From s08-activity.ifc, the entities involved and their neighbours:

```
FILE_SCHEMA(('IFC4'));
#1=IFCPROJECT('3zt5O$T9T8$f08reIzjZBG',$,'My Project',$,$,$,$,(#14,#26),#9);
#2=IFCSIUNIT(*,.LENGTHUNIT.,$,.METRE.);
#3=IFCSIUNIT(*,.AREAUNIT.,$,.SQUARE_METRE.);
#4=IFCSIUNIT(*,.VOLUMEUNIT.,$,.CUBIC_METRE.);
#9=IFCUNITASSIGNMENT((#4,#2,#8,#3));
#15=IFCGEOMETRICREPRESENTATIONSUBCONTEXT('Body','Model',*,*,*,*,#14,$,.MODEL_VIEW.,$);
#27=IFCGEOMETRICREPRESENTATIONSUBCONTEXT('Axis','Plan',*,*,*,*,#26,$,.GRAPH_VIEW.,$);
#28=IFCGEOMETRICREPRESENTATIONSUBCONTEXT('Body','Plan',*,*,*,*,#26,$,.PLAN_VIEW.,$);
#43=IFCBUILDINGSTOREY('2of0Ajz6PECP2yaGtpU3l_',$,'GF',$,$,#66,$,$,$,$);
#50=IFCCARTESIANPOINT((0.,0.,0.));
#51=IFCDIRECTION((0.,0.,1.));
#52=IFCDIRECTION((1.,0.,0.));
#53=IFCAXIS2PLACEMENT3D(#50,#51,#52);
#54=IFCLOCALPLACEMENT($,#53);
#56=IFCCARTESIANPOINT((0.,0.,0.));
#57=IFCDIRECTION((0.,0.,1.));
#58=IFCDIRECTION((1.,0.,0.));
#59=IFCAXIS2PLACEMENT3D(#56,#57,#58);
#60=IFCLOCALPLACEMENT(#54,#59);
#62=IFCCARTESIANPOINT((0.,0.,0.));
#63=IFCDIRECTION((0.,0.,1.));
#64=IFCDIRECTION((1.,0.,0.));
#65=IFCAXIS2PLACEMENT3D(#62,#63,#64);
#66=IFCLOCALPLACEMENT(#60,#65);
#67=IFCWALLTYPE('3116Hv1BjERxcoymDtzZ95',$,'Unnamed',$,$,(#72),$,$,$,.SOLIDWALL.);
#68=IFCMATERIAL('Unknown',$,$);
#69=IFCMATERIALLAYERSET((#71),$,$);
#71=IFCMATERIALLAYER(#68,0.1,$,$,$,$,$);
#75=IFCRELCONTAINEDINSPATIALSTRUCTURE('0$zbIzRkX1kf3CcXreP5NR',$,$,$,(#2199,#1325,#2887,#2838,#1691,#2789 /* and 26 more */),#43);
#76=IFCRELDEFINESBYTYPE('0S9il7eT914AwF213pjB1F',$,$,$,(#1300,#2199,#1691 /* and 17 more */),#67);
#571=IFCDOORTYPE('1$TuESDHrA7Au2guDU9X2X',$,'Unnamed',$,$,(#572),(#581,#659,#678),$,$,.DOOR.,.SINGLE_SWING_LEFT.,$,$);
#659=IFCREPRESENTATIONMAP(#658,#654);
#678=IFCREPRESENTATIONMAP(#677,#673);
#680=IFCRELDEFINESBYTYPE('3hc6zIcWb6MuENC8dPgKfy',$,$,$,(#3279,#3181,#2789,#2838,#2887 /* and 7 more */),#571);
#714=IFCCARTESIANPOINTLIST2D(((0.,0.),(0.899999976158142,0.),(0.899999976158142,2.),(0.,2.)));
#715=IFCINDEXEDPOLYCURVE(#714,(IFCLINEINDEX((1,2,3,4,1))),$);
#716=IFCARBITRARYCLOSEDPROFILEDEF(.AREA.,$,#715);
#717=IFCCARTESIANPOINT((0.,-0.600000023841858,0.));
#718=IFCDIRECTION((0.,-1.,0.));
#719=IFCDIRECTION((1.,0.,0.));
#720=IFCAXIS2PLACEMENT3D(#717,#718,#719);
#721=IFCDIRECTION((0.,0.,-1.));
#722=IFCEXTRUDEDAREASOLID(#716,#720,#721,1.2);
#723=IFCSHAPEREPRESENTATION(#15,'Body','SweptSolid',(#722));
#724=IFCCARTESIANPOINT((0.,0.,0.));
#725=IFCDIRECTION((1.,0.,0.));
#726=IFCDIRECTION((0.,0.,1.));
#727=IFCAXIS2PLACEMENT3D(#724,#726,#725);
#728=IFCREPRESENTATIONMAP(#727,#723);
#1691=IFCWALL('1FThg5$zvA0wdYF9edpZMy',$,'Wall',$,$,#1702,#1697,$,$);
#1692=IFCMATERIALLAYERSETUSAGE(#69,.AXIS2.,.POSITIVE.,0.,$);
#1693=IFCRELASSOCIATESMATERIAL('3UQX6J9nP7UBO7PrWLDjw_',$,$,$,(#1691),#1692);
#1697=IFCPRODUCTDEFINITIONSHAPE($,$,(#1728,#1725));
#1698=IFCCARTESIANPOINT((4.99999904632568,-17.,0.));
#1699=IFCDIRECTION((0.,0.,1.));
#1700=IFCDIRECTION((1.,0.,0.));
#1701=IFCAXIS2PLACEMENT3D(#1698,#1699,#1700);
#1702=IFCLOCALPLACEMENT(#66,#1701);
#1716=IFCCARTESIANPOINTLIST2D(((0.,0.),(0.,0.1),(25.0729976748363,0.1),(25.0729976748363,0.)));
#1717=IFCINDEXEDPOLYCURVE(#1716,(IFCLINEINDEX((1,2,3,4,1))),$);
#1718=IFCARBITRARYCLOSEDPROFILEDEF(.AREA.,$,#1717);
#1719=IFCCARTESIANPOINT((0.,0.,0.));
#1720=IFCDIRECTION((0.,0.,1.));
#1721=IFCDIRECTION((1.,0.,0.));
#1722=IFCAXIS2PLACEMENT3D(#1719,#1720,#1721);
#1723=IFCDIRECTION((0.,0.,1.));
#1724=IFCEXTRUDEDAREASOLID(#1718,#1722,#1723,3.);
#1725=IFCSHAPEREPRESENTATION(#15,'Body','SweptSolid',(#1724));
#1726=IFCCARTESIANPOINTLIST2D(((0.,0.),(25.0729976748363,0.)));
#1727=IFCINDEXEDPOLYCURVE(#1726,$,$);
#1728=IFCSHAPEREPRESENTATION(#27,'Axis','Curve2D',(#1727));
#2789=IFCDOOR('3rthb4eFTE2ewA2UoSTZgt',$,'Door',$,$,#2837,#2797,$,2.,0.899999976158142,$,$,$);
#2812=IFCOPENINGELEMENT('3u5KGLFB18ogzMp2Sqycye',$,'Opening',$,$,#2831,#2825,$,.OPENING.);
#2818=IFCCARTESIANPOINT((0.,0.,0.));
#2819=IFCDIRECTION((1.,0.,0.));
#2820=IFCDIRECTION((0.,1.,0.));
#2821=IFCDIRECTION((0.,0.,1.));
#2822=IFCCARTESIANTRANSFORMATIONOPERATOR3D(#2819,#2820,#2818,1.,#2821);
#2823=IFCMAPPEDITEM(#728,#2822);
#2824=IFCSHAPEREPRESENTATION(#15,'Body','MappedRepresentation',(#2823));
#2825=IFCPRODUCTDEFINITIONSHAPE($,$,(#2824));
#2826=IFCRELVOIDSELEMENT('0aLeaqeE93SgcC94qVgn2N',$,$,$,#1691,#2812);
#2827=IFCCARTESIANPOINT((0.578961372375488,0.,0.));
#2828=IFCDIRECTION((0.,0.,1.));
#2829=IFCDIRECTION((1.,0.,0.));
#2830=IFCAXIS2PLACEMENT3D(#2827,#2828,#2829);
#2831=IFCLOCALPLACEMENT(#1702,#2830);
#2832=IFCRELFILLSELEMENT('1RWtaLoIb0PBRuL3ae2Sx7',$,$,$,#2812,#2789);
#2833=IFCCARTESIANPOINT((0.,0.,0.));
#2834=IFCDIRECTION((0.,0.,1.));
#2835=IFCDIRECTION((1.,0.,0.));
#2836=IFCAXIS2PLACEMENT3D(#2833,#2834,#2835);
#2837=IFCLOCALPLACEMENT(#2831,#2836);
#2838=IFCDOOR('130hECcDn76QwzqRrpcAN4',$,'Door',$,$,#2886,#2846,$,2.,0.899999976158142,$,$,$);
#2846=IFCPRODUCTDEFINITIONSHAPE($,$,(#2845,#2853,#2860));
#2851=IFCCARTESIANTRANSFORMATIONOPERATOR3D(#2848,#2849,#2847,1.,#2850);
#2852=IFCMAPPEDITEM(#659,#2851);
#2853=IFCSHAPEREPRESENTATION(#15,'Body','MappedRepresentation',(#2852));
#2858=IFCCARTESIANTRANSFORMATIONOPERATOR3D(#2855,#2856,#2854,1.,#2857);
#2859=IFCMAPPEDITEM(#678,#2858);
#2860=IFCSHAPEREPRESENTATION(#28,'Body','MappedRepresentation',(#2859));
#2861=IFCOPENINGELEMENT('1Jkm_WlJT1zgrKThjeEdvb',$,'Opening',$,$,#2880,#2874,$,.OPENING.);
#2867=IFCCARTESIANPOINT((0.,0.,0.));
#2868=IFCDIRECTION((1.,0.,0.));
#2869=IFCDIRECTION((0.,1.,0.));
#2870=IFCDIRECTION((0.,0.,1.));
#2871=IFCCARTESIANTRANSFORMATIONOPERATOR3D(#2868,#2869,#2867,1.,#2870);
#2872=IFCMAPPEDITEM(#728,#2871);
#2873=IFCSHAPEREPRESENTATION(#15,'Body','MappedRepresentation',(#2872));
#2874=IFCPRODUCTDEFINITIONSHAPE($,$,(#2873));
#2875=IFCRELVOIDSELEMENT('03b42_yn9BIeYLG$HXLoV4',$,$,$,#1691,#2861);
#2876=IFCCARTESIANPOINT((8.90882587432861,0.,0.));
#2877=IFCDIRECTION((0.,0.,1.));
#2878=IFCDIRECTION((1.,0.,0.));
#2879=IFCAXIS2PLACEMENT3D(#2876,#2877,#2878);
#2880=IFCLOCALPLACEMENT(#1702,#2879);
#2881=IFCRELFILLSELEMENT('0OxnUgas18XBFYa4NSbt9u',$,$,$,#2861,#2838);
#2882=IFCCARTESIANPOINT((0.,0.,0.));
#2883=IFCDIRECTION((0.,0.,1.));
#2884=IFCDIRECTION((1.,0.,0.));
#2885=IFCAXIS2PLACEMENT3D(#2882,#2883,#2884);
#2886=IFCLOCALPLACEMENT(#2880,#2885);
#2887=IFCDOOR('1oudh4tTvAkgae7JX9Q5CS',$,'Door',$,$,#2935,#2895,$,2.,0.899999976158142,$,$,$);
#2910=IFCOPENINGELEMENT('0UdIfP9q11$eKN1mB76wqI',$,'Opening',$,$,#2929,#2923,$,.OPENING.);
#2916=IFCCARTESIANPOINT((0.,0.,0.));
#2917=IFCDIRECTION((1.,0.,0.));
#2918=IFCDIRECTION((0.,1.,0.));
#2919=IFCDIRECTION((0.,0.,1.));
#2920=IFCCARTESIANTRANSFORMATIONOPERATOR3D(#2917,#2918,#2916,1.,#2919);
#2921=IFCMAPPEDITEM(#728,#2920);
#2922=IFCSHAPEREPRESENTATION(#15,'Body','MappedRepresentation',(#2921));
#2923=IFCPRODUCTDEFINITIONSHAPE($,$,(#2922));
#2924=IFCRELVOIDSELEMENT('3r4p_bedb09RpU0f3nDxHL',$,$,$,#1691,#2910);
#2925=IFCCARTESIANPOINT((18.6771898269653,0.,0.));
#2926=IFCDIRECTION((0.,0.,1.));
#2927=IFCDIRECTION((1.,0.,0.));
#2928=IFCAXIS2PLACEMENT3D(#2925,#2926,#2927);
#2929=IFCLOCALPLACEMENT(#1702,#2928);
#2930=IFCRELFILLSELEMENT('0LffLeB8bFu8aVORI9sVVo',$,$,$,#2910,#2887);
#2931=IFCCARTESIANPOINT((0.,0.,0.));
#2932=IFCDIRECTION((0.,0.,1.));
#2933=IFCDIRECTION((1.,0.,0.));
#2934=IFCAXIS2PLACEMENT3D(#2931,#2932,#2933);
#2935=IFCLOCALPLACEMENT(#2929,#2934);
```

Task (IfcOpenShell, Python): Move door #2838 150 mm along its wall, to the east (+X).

```python
import ifcopenshell
import ifcopenshell.api.geometry
import ifcopenshell.util.placement

model = ifcopenshell.open("s08-activity.ifc")

door = model.by_guid("130hECcDn76QwzqRrpcAN4")
opening = door.FillsVoids[0].RelatingOpeningElement
wall = opening.VoidsElements[0].RelatingBuildingElement

wall_matrix = ifcopenshell.util.placement.get_local_placement(wall.ObjectPlacement)
shift = wall_matrix[:3, 0] * 0.15
before = ifcopenshell.util.placement.get_local_placement(door.ObjectPlacement)[:3, 3].copy()

# The door is placed relative to its opening, so it follows when the opening moves.
matrix = ifcopenshell.util.placement.get_local_placement(opening.ObjectPlacement)
matrix[:3, 3] += shift
ifcopenshell.api.geometry.edit_object_placement(
    model, product=opening, matrix=matrix, is_si=False, should_transform_children=True
)

after = ifcopenshell.util.placement.get_local_placement(door.ObjectPlacement)[:3, 3]
print("door moved by", (after - before).round(3) + 0.0)

model.write("s08-activity_edited.ifc")
```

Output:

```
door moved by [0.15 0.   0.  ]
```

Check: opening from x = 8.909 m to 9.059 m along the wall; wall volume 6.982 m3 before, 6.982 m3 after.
